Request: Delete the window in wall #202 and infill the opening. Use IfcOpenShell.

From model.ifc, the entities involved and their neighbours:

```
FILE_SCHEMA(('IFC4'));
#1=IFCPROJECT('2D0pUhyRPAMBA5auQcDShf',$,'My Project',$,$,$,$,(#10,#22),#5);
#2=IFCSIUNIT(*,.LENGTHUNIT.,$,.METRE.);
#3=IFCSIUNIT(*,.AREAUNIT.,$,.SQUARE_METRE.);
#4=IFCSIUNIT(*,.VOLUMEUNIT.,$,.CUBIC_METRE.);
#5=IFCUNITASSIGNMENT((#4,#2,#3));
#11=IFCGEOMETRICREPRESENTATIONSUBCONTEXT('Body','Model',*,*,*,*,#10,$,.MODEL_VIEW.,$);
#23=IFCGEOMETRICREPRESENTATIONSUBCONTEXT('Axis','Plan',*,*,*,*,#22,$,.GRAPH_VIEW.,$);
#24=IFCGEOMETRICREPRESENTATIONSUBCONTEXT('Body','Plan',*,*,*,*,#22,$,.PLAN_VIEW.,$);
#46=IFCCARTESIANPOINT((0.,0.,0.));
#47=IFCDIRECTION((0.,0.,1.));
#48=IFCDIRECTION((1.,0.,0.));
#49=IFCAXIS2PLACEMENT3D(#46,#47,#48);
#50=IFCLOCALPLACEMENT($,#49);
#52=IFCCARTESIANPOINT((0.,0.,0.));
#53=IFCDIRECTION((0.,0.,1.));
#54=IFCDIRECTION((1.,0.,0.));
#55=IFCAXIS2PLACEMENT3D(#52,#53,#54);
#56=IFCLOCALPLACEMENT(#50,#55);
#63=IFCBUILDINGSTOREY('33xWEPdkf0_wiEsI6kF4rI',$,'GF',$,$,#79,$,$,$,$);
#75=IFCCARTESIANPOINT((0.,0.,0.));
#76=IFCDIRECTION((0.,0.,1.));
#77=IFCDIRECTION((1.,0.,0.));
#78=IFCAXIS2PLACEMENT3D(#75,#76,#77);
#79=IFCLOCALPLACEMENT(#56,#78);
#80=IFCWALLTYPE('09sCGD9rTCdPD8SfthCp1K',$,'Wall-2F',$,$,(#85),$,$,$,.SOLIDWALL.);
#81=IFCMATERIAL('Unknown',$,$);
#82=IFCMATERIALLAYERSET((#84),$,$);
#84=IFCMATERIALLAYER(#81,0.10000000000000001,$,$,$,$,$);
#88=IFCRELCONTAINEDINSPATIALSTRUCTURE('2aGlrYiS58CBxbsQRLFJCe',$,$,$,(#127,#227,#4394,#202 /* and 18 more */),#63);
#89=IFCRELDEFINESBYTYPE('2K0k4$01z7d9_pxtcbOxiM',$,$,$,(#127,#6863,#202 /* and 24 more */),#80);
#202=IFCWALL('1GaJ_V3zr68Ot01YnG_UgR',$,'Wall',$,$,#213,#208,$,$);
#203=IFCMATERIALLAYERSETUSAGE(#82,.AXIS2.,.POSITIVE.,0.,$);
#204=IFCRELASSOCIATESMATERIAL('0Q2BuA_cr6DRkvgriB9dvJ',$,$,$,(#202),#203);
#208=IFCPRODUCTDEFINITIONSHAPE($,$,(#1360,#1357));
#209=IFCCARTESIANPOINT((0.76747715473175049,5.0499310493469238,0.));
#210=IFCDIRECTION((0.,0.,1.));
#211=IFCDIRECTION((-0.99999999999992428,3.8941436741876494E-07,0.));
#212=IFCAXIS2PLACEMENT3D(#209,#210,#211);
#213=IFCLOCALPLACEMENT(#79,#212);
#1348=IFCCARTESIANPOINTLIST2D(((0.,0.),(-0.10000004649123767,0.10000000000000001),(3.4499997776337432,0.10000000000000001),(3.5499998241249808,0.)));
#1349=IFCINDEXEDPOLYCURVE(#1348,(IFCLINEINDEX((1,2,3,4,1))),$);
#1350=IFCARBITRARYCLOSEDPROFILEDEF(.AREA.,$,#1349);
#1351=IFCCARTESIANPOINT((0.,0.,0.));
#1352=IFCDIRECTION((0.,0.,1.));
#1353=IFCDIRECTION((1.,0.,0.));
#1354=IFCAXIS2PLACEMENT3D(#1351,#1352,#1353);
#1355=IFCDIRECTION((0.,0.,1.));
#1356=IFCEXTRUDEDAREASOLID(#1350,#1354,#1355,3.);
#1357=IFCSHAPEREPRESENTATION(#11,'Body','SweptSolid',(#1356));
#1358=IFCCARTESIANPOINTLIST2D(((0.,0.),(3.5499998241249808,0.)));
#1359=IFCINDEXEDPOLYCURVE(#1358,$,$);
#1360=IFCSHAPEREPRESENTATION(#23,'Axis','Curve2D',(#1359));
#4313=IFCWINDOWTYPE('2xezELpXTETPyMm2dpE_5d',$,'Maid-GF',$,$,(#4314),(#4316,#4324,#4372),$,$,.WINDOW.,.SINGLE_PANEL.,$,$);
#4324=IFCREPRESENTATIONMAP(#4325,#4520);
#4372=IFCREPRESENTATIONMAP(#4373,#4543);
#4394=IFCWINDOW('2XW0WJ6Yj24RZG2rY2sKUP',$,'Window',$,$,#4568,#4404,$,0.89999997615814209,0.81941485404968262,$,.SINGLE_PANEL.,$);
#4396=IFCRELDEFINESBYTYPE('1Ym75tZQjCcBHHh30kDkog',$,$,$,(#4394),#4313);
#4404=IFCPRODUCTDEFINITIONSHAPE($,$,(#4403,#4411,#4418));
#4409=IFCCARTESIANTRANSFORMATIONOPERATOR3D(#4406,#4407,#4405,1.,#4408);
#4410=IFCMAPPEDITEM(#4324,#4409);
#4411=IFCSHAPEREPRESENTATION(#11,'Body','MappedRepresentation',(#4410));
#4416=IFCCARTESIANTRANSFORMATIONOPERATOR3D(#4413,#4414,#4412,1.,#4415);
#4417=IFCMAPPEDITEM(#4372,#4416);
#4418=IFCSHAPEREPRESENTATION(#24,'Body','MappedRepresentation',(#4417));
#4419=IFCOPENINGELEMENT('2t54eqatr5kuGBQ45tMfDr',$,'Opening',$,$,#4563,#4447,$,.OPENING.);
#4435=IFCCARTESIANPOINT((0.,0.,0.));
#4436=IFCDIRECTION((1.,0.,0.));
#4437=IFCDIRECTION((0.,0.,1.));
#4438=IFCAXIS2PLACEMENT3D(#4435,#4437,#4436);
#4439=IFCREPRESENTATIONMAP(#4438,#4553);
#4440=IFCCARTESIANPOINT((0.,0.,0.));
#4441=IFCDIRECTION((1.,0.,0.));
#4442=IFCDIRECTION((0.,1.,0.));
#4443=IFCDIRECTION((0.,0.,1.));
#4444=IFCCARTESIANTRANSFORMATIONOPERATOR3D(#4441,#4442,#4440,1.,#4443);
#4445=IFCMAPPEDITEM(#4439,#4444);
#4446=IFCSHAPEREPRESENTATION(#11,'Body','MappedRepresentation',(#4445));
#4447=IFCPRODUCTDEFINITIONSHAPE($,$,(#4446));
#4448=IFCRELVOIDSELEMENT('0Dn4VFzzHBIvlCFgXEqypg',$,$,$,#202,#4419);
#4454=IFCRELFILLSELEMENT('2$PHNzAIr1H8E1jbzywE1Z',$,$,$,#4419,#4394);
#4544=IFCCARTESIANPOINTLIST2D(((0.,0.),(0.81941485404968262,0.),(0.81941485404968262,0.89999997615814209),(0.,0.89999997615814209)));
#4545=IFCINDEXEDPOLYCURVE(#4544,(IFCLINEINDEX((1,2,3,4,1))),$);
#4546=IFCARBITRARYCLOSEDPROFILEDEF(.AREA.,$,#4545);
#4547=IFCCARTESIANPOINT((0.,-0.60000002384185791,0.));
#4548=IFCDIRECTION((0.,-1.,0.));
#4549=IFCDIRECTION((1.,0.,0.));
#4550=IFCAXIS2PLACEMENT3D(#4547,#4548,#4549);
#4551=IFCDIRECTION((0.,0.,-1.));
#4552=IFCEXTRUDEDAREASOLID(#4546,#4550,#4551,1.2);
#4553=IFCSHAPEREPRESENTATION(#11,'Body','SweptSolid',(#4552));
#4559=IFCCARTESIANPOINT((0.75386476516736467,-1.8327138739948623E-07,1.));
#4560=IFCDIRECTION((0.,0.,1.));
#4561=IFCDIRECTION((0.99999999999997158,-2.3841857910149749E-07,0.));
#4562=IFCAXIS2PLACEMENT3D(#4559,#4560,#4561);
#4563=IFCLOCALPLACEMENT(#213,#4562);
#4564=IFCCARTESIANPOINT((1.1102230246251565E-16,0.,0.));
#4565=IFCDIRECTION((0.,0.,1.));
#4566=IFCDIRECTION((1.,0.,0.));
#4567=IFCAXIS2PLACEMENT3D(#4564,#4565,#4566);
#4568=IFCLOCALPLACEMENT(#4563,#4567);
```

```python
import ifcopenshell
import ifcopenshell.api.feature
import ifcopenshell.api.root
import ifcopenshell.geom
import ifcopenshell.util.shape

model = ifcopenshell.open("model.ifc")
settings = ifcopenshell.geom.settings()


def volume(element):
    """Net volume in cubic metres, openings subtracted."""
    shape = ifcopenshell.geom.create_shape(settings, element)
    return ifcopenshell.util.shape.get_volume(shape.geometry)


window = model.by_guid("2XW0WJ6Yj24RZG2rY2sKUP")
opening = window.FillsVoids[0].RelatingOpeningElement
wall = opening.VoidsElements[0].RelatingBuildingElement
before = volume(wall)

ifcopenshell.api.root.remove_product(model, product=window)
ifcopenshell.api.feature.remove_feature(model, feature=opening)

after = volume(wall)

print(f"wall volume {before:.3f} -> {after:.3f} m3")

model.write("model_updated.ifc")
```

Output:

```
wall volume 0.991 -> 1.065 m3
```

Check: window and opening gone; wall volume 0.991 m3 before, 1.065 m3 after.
